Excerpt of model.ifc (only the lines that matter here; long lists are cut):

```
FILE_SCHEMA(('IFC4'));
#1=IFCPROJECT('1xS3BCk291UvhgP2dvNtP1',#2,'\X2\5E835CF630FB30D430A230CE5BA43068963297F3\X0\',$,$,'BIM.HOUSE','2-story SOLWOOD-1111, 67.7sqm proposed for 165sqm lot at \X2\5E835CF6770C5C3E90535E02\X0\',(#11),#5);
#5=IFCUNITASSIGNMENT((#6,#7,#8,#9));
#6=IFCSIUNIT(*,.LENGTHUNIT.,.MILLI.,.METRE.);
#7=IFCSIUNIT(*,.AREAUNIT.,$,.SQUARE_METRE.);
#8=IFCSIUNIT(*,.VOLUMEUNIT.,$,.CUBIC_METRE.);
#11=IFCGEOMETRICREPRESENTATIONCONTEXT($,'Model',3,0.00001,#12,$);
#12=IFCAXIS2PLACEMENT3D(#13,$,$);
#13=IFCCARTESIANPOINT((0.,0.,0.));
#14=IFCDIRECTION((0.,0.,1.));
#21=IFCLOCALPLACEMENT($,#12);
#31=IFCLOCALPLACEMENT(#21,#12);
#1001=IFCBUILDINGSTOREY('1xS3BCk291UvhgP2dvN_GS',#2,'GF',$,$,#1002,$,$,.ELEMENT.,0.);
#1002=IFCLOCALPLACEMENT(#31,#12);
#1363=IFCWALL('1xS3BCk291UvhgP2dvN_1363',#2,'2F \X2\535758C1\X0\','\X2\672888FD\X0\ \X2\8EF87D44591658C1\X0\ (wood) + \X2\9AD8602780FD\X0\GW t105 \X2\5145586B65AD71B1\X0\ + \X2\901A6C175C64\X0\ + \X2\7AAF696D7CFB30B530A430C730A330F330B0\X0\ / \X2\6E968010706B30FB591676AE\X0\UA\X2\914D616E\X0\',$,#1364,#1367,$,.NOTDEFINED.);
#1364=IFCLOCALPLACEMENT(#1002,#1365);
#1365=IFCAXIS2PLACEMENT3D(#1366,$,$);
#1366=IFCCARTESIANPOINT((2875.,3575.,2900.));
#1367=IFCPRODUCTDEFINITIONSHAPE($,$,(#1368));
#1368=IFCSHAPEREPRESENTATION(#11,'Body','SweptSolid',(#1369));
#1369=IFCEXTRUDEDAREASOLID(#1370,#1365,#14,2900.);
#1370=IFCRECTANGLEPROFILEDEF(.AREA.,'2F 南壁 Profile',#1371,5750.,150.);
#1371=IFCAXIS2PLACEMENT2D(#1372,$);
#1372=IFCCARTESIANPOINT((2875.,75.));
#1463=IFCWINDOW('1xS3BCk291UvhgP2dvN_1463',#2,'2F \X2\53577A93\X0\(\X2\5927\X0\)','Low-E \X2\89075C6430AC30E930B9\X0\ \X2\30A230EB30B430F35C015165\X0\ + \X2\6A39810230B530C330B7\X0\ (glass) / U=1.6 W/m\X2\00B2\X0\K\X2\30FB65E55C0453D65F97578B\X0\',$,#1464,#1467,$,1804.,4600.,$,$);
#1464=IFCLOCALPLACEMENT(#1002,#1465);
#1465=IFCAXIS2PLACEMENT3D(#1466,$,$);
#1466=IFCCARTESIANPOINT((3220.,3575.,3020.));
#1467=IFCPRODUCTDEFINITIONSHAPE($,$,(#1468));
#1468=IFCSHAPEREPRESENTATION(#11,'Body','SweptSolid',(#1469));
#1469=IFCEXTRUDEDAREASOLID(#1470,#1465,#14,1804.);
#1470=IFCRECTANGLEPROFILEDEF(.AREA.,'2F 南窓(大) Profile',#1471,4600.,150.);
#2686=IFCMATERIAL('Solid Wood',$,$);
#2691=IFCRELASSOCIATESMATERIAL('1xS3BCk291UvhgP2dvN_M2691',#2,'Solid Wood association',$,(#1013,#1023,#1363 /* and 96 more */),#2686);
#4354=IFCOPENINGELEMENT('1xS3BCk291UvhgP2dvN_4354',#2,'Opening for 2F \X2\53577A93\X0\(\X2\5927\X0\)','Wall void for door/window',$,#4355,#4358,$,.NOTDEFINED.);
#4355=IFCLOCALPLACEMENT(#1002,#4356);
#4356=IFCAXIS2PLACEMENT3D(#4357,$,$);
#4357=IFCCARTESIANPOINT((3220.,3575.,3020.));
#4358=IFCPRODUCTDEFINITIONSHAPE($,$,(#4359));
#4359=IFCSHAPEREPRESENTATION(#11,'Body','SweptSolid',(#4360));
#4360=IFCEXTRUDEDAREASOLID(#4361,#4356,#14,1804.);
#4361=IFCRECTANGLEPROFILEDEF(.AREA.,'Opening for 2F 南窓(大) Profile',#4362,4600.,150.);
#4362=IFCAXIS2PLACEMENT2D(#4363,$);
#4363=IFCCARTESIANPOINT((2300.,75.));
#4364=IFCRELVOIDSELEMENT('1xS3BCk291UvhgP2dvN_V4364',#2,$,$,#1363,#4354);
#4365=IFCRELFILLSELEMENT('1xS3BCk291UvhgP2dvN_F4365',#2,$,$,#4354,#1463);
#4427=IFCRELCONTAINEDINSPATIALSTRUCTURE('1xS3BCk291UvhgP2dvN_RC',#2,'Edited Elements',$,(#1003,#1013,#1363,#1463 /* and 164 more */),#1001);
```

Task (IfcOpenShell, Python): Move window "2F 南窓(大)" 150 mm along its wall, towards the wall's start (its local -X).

```python
import ifcopenshell
import ifcopenshell.api.geometry
import ifcopenshell.util.placement
import ifcopenshell.util.unit

model = ifcopenshell.open("model.ifc")
unit_scale = ifcopenshell.util.unit.calculate_unit_scale(model)

window = model.by_id(1463)
opening = window.FillsVoids[0].RelatingOpeningElement
wall = opening.VoidsElements[0].RelatingBuildingElement

wall_matrix = ifcopenshell.util.placement.get_local_placement(wall.ObjectPlacement)
shift = wall_matrix[:3, 0] * -0.15 / unit_scale
before = ifcopenshell.util.placement.get_local_placement(window.ObjectPlacement)[:3, 3].copy()

# The window is not placed relative to its opening, so move both.
for product in (opening, window):
    matrix = ifcopenshell.util.placement.get_local_placement(product.ObjectPlacement)
    matrix[:3, 3] += shift
    ifcopenshell.api.geometry.edit_object_placement(model, product=product, matrix=matrix, is_si=False)

after = ifcopenshell.util.placement.get_local_placement(window.ObjectPlacement)[:3, 3]
print("window moved by", (after - before).round(3) + 0.0)

model.write("model_updated.ifc")
```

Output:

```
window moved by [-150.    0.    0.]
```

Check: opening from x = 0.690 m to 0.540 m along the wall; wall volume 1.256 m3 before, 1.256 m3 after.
